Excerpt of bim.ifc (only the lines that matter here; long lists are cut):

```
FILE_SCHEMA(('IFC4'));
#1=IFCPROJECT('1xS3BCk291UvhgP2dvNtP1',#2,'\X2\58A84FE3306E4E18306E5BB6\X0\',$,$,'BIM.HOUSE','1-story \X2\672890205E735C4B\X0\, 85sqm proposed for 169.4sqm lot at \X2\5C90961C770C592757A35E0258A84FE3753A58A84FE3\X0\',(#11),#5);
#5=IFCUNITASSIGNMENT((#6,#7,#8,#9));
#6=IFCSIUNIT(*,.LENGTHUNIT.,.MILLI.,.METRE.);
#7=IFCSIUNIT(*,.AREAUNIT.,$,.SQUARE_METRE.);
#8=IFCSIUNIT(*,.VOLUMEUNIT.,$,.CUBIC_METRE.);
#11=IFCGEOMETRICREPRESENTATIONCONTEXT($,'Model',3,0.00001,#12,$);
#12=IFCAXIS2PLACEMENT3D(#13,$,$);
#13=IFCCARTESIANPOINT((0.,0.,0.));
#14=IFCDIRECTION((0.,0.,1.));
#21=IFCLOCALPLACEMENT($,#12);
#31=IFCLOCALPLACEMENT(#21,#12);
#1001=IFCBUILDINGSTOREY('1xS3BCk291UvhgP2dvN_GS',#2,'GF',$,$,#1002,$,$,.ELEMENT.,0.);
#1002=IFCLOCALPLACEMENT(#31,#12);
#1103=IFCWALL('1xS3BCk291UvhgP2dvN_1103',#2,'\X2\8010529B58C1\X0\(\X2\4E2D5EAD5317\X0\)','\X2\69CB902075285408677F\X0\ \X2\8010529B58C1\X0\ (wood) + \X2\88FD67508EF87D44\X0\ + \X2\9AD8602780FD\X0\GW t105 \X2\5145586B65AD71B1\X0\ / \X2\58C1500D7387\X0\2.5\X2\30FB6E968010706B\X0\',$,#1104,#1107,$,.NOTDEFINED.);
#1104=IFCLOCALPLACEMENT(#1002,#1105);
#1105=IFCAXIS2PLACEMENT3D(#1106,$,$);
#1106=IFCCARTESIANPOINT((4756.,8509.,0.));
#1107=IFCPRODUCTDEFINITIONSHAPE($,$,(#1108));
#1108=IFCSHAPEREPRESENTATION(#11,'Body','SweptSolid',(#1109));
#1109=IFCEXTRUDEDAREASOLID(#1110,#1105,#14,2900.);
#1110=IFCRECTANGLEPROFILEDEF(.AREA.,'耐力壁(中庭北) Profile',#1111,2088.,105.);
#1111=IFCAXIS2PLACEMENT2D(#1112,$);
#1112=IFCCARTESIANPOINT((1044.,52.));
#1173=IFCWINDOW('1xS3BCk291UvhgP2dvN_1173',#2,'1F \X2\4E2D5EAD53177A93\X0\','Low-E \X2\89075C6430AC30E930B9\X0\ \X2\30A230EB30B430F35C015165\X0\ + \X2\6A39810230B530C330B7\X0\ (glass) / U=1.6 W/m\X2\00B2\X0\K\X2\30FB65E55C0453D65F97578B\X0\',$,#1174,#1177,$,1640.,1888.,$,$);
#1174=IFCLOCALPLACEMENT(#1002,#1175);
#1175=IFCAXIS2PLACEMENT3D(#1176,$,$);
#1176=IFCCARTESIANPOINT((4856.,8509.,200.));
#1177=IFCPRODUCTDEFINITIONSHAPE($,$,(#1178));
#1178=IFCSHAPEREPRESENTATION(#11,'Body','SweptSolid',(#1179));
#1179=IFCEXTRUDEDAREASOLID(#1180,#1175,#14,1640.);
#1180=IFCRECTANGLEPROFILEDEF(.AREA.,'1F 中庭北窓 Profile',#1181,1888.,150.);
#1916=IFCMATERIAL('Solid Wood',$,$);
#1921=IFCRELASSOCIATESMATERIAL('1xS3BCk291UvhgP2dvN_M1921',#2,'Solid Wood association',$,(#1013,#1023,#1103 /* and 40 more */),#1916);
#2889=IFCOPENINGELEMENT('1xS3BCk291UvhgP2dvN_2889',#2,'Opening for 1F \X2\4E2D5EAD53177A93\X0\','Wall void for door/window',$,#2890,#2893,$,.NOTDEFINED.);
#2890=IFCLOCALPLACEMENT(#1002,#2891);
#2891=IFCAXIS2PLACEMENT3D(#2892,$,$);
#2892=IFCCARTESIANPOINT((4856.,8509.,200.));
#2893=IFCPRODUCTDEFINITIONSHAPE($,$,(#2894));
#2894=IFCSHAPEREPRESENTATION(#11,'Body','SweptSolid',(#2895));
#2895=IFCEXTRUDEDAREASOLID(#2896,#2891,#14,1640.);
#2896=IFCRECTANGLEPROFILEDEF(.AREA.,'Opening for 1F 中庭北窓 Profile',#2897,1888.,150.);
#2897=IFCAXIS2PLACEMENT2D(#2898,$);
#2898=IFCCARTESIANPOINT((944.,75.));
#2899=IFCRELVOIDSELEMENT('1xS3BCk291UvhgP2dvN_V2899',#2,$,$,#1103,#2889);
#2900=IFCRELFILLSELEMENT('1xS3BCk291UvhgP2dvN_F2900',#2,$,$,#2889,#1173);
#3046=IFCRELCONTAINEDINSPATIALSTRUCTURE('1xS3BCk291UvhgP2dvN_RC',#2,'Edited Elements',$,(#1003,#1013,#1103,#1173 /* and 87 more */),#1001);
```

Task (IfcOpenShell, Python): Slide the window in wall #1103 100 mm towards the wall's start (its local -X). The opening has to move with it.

```python
import ifcopenshell
import ifcopenshell.api.geometry
import ifcopenshell.util.placement
import ifcopenshell.util.unit

model = ifcopenshell.open("bim.ifc")
unit_scale = ifcopenshell.util.unit.calculate_unit_scale(model)

window = model.by_id(1173)
opening = window.FillsVoids[0].RelatingOpeningElement
wall = opening.VoidsElements[0].RelatingBuildingElement

wall_matrix = ifcopenshell.util.placement.get_local_placement(wall.ObjectPlacement)
shift = wall_matrix[:3, 0] * -0.1 / unit_scale
before = ifcopenshell.util.placement.get_local_placement(window.ObjectPlacement)[:3, 3].copy()

# The window is not placed relative to its opening, so move both.
for product in (opening, window):
    matrix = ifcopenshell.util.placement.get_local_placement(product.ObjectPlacement)
    matrix[:3, 3] += shift
    ifcopenshell.api.geometry.edit_object_placement(model, product=product, matrix=matrix, is_si=False)

after = ifcopenshell.util.placement.get_local_placement(window.ObjectPlacement)[:3, 3]
print("window moved by", (after - before).round(3) + 0.0)

model.write("bim_edited.ifc")
```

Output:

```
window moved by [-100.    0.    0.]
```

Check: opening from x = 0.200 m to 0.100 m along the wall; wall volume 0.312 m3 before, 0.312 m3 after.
